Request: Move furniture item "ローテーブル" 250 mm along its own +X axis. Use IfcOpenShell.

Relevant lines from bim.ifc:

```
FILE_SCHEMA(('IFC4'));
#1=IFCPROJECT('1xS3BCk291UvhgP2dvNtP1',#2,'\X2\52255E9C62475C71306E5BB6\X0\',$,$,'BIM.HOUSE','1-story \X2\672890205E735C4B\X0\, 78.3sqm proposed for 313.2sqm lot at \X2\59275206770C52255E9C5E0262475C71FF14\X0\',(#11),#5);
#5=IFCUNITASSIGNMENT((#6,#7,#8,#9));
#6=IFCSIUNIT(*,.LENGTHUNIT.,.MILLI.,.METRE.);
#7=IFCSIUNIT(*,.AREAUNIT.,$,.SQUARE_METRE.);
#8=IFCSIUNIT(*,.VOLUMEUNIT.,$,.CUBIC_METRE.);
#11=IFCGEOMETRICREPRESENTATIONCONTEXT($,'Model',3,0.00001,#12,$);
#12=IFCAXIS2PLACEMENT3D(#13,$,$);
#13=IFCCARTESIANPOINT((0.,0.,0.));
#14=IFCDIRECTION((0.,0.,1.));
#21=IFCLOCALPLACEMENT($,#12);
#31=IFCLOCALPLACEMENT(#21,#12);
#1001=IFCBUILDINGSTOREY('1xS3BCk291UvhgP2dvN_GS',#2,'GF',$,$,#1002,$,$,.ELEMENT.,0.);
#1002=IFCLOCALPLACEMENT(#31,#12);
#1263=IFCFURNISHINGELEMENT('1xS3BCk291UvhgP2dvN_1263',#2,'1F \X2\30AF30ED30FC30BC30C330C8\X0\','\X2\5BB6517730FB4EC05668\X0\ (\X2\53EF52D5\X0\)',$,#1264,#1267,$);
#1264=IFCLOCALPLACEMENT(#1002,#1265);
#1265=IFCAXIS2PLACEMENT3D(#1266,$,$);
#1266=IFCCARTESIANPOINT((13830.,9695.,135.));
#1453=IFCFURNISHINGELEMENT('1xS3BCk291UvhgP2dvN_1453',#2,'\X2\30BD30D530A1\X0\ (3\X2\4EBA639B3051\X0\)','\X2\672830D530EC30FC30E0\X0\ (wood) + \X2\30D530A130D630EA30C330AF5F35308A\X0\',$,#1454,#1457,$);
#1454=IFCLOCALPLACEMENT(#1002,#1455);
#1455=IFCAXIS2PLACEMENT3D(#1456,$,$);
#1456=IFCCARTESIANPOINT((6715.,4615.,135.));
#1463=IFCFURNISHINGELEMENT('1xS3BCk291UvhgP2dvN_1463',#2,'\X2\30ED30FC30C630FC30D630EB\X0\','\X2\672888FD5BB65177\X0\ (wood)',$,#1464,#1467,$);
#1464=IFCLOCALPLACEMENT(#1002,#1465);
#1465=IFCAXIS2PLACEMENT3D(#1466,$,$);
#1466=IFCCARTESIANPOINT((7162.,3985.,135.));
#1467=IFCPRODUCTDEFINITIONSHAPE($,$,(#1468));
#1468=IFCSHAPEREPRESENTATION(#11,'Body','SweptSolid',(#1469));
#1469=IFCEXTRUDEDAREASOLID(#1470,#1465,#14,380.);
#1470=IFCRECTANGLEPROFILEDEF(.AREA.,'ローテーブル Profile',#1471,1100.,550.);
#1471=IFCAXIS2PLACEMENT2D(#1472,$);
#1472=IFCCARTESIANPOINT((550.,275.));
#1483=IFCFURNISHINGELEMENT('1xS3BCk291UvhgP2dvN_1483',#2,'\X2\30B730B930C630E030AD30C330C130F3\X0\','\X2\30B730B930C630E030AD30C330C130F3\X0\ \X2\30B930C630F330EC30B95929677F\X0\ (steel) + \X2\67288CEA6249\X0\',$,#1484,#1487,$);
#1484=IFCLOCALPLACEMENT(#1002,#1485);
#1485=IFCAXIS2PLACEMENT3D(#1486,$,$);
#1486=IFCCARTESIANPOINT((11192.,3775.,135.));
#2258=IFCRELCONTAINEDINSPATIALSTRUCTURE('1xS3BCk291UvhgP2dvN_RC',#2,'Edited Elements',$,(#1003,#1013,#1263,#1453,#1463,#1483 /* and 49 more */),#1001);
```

```python
import ifcopenshell
import ifcopenshell.api.geometry
import ifcopenshell.util.placement

model = ifcopenshell.open("bim.ifc")

item = model.by_guid("1xS3BCk291UvhgP2dvN_1463")
matrix = ifcopenshell.util.placement.get_local_placement(item.ObjectPlacement)
matrix[:3, 3] += matrix[:3, 0] * 250.0
ifcopenshell.api.geometry.edit_object_placement(model, product=item, matrix=matrix, is_si=False)

print(ifcopenshell.util.placement.get_local_placement(item.ObjectPlacement).round(3) + 0.0)

model.write("bim_rev.ifc")
```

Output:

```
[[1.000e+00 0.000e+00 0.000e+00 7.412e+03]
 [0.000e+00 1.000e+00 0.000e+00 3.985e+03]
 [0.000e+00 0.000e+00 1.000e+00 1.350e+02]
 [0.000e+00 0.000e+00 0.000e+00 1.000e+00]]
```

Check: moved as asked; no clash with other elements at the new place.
